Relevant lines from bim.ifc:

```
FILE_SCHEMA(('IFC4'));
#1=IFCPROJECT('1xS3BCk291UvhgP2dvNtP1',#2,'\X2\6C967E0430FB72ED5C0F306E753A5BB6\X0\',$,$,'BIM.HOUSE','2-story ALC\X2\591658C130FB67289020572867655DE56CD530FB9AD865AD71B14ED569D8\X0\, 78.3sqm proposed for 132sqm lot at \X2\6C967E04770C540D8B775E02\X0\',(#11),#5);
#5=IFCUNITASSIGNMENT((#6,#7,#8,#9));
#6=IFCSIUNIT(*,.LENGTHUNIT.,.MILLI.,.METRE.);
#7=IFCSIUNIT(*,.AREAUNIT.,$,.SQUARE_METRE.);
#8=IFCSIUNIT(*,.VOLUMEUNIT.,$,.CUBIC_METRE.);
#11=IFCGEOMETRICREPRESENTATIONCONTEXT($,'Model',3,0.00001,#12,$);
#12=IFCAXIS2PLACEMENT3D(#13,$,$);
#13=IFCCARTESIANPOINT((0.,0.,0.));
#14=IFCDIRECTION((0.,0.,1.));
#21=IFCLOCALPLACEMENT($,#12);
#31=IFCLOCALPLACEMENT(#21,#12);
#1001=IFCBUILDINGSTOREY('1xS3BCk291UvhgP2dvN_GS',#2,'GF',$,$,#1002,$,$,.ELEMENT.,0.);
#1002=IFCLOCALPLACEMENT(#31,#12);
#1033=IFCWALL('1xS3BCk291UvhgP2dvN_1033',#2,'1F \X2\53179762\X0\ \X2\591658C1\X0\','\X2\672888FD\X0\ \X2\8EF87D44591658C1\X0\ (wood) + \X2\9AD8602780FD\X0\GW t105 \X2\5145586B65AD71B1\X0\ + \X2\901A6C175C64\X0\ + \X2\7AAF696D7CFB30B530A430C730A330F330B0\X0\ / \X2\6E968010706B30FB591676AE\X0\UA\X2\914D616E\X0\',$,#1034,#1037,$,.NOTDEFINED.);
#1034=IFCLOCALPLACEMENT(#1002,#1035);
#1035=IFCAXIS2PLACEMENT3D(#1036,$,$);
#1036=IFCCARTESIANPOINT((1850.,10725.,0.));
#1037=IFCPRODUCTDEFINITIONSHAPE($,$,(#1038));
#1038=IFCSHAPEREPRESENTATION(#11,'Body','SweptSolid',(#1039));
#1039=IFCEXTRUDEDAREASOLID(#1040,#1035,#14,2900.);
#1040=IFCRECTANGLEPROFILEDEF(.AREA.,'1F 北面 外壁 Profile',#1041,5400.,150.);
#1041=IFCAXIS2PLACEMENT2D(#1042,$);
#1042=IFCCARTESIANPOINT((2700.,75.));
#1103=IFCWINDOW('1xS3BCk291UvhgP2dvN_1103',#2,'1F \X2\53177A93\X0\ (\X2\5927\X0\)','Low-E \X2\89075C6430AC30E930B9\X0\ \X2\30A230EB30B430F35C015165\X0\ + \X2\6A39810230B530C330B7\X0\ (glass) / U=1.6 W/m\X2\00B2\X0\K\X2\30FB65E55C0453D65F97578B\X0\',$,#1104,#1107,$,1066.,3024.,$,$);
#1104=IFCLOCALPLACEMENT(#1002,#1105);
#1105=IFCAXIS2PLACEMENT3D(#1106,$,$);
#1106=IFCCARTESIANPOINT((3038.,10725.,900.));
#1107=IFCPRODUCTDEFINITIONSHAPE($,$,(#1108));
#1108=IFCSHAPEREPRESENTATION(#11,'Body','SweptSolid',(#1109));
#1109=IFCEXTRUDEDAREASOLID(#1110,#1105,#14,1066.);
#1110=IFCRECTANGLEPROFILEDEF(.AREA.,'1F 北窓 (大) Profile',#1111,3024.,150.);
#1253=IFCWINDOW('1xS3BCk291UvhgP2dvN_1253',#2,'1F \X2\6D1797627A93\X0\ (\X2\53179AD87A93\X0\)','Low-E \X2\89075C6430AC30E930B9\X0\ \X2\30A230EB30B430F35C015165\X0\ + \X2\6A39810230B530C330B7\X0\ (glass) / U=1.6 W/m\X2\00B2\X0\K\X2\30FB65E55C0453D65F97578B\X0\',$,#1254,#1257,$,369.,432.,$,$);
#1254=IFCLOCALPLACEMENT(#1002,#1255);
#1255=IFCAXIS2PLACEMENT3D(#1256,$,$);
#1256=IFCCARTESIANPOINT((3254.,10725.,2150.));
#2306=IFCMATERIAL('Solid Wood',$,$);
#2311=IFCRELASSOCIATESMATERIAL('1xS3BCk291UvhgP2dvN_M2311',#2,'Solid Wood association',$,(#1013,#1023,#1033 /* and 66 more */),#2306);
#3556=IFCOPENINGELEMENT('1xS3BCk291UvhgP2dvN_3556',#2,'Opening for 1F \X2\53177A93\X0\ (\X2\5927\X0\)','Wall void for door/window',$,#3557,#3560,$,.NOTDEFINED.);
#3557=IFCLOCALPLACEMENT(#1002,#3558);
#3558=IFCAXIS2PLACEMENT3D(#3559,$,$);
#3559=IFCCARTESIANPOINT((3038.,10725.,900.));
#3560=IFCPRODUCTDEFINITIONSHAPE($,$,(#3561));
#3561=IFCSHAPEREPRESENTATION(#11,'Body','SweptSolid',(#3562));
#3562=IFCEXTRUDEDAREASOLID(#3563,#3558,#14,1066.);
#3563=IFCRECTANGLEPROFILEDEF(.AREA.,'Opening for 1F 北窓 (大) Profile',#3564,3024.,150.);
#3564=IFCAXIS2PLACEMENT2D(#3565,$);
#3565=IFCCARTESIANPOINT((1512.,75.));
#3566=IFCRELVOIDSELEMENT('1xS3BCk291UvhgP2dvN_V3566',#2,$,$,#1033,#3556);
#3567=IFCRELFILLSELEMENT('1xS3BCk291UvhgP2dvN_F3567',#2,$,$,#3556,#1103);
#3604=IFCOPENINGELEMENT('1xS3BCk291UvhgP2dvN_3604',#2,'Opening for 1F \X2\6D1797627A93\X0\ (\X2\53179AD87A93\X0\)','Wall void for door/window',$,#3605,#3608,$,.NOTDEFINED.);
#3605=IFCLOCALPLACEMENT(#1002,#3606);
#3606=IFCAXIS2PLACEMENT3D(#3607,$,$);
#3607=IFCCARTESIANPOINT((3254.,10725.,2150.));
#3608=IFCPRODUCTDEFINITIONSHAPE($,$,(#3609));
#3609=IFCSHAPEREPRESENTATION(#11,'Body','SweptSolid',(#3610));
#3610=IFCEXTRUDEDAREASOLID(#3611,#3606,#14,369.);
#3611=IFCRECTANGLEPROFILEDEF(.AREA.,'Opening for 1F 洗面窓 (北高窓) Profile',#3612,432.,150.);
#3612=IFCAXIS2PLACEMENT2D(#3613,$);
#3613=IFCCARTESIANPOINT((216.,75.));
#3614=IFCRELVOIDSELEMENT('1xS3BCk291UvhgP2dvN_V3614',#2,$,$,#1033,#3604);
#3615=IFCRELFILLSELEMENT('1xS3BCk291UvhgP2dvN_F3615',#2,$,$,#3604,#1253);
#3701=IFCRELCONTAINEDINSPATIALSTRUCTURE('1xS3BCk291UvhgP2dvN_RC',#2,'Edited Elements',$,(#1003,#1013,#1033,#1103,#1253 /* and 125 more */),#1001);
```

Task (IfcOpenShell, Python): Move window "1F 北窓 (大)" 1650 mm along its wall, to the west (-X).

```python
import ifcopenshell
import ifcopenshell.api.geometry
import ifcopenshell.util.placement
import ifcopenshell.util.unit

model = ifcopenshell.open("bim.ifc")
unit_scale = ifcopenshell.util.unit.calculate_unit_scale(model)

window = model.by_guid("1xS3BCk291UvhgP2dvN_1103")
opening = window.FillsVoids[0].RelatingOpeningElement
wall = opening.VoidsElements[0].RelatingBuildingElement

wall_matrix = ifcopenshell.util.placement.get_local_placement(wall.ObjectPlacement)
shift = wall_matrix[:3, 0] * -1.65 / unit_scale
before = ifcopenshell.util.placement.get_local_placement(window.ObjectPlacement)[:3, 3].copy()

# The window is not placed relative to its opening, so move both.
for product in (opening, window):
    matrix = ifcopenshell.util.placement.get_local_placement(product.ObjectPlacement)
    matrix[:3, 3] += shift
    ifcopenshell.api.geometry.edit_object_placement(model, product=product, matrix=matrix, is_si=False)

after = ifcopenshell.util.placement.get_local_placement(window.ObjectPlacement)[:3, 3]
print("window moved by", (after - before).round(3) + 0.0)

model.write("bim_edited.ifc")
```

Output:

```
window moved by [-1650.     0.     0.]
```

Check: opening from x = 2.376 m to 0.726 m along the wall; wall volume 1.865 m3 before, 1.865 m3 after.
